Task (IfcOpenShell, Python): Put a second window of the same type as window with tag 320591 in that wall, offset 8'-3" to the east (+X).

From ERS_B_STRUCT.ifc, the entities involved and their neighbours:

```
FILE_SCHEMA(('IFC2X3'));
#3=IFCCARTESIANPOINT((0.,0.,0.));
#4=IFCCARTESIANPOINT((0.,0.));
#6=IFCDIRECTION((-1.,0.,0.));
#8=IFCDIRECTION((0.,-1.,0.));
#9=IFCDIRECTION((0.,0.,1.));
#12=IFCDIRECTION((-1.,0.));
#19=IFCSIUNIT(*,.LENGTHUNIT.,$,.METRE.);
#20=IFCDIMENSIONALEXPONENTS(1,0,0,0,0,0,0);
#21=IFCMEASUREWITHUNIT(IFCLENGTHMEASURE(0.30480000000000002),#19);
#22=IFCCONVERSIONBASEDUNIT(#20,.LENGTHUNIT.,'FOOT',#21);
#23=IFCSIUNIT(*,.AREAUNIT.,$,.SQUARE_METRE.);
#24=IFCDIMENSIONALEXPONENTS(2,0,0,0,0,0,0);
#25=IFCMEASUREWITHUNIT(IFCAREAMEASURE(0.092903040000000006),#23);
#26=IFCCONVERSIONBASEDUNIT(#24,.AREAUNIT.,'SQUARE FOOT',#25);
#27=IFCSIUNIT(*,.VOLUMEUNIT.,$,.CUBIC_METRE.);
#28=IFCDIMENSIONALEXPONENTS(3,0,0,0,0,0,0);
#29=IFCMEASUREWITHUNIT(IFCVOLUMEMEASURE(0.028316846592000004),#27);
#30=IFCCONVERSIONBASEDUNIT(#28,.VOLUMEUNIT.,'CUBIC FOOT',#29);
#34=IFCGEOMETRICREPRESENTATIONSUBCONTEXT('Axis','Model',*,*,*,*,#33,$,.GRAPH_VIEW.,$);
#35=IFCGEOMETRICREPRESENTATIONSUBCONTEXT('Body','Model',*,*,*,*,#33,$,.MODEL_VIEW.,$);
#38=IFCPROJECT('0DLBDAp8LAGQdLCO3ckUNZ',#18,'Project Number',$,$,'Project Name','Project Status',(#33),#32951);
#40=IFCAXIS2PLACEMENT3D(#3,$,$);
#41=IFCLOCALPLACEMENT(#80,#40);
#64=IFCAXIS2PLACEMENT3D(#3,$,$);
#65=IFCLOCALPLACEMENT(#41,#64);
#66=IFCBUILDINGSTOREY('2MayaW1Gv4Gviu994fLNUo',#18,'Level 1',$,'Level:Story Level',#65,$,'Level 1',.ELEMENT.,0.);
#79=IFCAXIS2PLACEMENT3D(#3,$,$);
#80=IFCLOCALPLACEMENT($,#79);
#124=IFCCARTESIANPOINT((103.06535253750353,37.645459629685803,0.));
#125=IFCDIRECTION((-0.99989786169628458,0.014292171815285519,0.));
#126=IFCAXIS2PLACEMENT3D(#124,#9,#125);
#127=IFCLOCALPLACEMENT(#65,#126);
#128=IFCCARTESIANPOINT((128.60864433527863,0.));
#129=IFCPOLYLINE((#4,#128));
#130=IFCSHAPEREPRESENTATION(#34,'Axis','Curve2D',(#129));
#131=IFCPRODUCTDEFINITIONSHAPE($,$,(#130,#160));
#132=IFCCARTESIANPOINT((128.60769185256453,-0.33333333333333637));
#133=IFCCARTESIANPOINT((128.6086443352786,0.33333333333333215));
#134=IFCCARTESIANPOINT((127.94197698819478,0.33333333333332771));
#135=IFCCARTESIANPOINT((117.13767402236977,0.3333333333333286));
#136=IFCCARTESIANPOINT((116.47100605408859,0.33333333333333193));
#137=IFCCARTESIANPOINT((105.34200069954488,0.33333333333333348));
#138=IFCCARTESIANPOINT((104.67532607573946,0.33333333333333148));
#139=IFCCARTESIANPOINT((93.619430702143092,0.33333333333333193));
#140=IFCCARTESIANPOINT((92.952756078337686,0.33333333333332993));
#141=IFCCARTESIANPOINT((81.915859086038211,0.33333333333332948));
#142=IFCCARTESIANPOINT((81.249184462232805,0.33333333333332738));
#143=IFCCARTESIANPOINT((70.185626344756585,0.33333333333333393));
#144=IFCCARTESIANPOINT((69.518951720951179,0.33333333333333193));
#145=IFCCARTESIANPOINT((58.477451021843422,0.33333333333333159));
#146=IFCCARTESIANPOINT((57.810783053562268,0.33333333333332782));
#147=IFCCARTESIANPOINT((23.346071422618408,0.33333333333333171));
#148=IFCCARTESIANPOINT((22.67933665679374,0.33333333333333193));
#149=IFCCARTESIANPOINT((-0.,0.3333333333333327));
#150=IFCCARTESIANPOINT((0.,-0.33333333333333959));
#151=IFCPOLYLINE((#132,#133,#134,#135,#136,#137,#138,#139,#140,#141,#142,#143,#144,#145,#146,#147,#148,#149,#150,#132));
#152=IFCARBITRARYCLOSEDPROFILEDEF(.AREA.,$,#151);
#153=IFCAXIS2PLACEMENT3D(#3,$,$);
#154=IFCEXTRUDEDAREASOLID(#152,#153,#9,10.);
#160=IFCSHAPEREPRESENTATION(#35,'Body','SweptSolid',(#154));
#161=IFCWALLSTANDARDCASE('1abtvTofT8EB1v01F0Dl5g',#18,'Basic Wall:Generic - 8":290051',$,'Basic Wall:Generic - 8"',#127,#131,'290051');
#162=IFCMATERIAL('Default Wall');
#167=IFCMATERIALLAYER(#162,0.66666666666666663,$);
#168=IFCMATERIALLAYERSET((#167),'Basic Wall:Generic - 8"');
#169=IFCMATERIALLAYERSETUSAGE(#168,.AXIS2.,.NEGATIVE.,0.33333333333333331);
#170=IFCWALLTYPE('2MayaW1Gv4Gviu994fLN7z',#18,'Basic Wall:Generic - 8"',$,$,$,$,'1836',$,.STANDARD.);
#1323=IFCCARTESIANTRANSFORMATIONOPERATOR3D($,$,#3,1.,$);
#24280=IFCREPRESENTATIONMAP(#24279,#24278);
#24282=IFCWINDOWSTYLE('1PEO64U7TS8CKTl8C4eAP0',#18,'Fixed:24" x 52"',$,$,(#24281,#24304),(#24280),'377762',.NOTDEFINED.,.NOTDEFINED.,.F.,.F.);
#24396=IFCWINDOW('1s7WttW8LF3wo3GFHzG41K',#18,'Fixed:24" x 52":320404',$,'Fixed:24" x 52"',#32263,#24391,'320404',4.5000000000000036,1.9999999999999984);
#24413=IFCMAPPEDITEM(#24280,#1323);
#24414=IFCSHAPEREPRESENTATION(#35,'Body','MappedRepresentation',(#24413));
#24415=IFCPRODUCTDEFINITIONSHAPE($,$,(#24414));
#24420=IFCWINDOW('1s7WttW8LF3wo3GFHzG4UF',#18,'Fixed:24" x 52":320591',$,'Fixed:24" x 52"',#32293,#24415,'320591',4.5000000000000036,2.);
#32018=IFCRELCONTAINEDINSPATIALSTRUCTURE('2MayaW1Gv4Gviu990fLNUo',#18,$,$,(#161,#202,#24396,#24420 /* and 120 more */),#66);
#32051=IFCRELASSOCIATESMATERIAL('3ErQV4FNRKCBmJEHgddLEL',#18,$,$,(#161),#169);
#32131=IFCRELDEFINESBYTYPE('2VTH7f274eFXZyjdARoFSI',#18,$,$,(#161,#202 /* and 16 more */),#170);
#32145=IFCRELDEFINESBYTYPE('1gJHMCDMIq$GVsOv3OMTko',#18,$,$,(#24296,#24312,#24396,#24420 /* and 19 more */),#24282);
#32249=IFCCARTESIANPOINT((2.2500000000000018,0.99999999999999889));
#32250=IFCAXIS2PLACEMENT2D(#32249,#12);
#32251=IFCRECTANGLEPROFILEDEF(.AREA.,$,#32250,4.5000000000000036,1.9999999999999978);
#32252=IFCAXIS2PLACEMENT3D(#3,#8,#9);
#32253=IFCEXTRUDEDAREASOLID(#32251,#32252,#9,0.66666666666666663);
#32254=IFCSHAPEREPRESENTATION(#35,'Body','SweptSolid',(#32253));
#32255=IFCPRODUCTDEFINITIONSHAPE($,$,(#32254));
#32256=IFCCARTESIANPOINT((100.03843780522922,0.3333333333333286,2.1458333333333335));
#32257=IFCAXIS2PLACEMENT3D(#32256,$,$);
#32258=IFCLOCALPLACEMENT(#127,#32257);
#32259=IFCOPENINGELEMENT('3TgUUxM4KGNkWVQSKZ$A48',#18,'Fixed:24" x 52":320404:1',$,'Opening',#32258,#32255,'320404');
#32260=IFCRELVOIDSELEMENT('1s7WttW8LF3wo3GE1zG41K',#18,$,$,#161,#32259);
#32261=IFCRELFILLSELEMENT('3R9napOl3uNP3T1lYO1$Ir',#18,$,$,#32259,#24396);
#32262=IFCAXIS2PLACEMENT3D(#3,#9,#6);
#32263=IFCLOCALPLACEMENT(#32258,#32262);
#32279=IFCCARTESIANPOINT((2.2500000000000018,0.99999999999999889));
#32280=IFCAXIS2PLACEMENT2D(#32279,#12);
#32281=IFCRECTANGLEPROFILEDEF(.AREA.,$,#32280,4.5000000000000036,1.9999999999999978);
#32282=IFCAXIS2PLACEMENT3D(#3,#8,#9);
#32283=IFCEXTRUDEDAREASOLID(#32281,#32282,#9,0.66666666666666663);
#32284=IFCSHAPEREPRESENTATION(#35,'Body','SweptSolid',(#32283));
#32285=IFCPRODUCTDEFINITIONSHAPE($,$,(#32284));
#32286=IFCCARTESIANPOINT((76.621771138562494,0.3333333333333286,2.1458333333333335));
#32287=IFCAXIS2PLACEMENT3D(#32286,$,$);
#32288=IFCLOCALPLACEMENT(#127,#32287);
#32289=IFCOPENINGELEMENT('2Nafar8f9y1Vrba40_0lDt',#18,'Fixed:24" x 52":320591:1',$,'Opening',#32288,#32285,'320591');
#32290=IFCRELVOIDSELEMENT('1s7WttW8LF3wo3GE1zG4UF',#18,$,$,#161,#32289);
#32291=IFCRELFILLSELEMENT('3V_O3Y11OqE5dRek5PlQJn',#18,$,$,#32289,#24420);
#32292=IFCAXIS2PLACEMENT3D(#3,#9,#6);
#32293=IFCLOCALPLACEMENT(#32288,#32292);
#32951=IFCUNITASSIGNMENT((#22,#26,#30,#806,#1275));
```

```python
import ifcopenshell
import ifcopenshell.api.feature
import ifcopenshell.api.geometry
import ifcopenshell.api.root
import ifcopenshell.geom
import ifcopenshell.util.element
import ifcopenshell.util.placement
import ifcopenshell.util.shape
import ifcopenshell.util.unit

model = ifcopenshell.open("ERS_B_STRUCT.ifc")
unit_scale = ifcopenshell.util.unit.calculate_unit_scale(model)
settings = ifcopenshell.geom.settings()


def volume(element):
    """Net volume in cubic metres, openings subtracted."""
    shape = ifcopenshell.geom.create_shape(settings, element)
    return ifcopenshell.util.shape.get_volume(shape.geometry)


def reuse_history(source, copy):
    """copy_class also copies each property set's owner history, people and application; keep the originals."""
    for rel in copy.IsDefinedBy:
        if rel.is_a("IfcRelDefinesByProperties") and (history := rel.RelatingPropertyDefinition.OwnerHistory):
            rel.RelatingPropertyDefinition.OwnerHistory = source.OwnerHistory
            ifcopenshell.util.element.remove_deep2(model, history)


window = model.by_guid("1s7WttW8LF3wo3GFHzG4UF")
opening = window.FillsVoids[0].RelatingOpeningElement
wall = opening.VoidsElements[0].RelatingBuildingElement
before = volume(wall)
shift = ifcopenshell.util.placement.get_local_placement(wall.ObjectPlacement)[:3, 0] * -99 * 0.0254 / unit_scale

# copy_class copies the void relationship, type, container and properties, but no geometry.
new_opening = ifcopenshell.api.root.copy_class(model, product=opening)
new_opening.Representation = ifcopenshell.util.element.copy_deep(
    model, opening.Representation, exclude=["IfcGeometricRepresentationContext", "IfcRepresentationMap"]
)
new_opening.Name = 'Fixed:24" x 52"'
new_opening.Tag = None
new_window = ifcopenshell.api.root.copy_class(model, product=window)
new_window.Representation = ifcopenshell.util.element.copy_deep(
    model, window.Representation, exclude=["IfcGeometricRepresentationContext", "IfcRepresentationMap"]
)
new_window.Name = 'Fixed:24" x 52"'
new_window.Tag = None
reuse_history(window, new_window)
fills = ifcopenshell.api.feature.add_filling(model, opening=new_opening, element=new_window)
fills.OwnerHistory = new_window.OwnerHistory  # required in IFC2X3

for old, new in ((opening, new_opening), (window, new_window)):
    matrix = ifcopenshell.util.placement.get_local_placement(old.ObjectPlacement)
    matrix[:3, 3] += shift
    ifcopenshell.api.geometry.edit_object_placement(model, product=new, matrix=matrix, is_si=False)

after = volume(wall)

print(f"wall volume {before:.3f} -> {after:.3f} m3")

model.write("ERS_B_STRUCT_rev.ifc")
```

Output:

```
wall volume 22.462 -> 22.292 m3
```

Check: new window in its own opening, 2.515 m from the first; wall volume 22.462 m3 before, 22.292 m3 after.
